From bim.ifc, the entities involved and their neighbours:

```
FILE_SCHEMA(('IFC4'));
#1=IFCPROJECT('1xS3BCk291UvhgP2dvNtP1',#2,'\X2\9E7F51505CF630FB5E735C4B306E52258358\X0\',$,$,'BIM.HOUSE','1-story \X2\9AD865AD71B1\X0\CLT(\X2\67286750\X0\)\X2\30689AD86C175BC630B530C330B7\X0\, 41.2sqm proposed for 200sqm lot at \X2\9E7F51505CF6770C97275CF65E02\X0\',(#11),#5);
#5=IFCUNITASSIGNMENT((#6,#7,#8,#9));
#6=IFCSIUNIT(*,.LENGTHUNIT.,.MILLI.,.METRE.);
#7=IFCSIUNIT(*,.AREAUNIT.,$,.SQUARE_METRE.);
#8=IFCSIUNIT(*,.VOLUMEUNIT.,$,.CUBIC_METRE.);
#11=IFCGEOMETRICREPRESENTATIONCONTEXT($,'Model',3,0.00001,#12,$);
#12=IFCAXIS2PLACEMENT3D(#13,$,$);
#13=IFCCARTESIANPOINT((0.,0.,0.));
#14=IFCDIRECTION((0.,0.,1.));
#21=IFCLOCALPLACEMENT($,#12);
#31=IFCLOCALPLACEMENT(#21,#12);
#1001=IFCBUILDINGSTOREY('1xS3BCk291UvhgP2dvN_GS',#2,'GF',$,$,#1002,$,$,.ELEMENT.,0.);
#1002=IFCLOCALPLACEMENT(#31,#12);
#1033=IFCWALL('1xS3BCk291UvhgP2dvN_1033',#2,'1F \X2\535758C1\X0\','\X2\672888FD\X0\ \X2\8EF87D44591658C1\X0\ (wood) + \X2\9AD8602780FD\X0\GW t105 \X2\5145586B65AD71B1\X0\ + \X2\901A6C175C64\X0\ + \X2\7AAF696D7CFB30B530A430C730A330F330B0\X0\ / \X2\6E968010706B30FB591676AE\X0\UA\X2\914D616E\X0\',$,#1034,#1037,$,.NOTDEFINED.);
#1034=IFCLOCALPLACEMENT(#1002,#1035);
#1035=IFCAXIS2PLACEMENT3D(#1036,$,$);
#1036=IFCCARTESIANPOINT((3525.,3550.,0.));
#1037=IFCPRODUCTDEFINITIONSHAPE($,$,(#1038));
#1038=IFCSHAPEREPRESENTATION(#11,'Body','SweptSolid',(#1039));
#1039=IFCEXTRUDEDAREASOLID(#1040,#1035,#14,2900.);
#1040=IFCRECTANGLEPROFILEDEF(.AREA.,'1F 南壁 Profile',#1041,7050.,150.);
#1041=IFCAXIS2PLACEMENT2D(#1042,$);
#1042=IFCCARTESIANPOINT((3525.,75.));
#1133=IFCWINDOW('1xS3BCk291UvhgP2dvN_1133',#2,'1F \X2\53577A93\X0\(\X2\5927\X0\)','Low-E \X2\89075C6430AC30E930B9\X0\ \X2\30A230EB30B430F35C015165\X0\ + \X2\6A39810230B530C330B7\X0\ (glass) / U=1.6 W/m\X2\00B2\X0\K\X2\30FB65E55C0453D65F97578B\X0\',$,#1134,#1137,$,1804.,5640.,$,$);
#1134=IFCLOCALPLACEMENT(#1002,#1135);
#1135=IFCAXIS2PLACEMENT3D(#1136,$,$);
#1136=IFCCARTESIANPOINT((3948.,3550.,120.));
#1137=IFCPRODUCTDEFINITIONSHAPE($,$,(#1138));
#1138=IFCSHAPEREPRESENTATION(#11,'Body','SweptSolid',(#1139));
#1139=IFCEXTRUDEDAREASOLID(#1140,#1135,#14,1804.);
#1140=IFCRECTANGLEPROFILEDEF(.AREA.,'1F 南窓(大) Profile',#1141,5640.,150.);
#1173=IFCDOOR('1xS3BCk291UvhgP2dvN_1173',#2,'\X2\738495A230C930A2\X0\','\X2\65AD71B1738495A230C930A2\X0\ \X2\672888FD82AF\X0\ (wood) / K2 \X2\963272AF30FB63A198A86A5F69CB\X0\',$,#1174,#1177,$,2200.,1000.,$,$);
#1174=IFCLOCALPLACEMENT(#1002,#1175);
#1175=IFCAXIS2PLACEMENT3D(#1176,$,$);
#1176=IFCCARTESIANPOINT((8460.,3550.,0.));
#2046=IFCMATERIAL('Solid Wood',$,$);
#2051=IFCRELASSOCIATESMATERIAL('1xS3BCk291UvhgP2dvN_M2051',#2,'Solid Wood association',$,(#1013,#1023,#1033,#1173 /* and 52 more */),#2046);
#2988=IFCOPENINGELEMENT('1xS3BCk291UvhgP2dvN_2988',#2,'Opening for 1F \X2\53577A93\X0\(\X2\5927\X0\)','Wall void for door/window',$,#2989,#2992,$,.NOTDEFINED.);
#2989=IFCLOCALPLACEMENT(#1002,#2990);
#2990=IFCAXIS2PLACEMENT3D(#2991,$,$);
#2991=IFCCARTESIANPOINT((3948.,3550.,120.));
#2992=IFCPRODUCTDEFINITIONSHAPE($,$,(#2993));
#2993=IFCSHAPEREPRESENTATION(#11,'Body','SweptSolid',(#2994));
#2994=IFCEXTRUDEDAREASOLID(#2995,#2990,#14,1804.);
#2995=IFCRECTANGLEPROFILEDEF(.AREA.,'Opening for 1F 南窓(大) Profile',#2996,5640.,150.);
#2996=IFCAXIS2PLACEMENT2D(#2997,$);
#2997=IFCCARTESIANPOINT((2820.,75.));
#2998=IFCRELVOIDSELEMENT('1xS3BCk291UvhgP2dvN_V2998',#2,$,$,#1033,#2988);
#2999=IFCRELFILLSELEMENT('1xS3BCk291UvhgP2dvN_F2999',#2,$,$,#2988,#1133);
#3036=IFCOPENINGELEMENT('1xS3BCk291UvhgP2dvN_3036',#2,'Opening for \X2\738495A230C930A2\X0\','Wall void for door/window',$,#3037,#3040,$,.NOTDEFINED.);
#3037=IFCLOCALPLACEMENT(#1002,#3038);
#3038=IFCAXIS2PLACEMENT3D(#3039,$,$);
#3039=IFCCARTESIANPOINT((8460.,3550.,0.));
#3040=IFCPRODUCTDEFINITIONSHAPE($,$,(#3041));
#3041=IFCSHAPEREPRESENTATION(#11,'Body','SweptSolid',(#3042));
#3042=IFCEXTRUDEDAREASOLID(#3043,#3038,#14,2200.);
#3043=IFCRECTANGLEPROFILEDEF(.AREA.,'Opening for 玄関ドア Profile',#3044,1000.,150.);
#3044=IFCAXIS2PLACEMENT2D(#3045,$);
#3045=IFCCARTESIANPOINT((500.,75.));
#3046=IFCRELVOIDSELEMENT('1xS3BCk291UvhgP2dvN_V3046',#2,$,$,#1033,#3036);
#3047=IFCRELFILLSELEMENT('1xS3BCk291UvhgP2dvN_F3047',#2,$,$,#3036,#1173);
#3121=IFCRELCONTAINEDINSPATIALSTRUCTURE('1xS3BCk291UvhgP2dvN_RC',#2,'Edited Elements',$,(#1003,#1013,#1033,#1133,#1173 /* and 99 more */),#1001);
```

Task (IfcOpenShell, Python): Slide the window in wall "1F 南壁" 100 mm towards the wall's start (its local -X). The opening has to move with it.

```python
import ifcopenshell
import ifcopenshell.api.geometry
import ifcopenshell.util.placement

model = ifcopenshell.open("bim.ifc")

window = model.by_guid("1xS3BCk291UvhgP2dvN_1133")
opening = window.FillsVoids[0].RelatingOpeningElement
wall = opening.VoidsElements[0].RelatingBuildingElement

wall_matrix = ifcopenshell.util.placement.get_local_placement(wall.ObjectPlacement)
shift = wall_matrix[:3, 0] * -100.0
before = ifcopenshell.util.placement.get_local_placement(window.ObjectPlacement)[:3, 3].copy()

# The window is not placed relative to its opening, so move both.
for product in (opening, window):
    matrix = ifcopenshell.util.placement.get_local_placement(product.ObjectPlacement)
    matrix[:3, 3] += shift
    ifcopenshell.api.geometry.edit_object_placement(model, product=product, matrix=matrix, is_si=False)

after = ifcopenshell.util.placement.get_local_placement(window.ObjectPlacement)[:3, 3]
print("window moved by", (after - before).round(3) + 0.0)

model.write("bim_edited.ifc")
```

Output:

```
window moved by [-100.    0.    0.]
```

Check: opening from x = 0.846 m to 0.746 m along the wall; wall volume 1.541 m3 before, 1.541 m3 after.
